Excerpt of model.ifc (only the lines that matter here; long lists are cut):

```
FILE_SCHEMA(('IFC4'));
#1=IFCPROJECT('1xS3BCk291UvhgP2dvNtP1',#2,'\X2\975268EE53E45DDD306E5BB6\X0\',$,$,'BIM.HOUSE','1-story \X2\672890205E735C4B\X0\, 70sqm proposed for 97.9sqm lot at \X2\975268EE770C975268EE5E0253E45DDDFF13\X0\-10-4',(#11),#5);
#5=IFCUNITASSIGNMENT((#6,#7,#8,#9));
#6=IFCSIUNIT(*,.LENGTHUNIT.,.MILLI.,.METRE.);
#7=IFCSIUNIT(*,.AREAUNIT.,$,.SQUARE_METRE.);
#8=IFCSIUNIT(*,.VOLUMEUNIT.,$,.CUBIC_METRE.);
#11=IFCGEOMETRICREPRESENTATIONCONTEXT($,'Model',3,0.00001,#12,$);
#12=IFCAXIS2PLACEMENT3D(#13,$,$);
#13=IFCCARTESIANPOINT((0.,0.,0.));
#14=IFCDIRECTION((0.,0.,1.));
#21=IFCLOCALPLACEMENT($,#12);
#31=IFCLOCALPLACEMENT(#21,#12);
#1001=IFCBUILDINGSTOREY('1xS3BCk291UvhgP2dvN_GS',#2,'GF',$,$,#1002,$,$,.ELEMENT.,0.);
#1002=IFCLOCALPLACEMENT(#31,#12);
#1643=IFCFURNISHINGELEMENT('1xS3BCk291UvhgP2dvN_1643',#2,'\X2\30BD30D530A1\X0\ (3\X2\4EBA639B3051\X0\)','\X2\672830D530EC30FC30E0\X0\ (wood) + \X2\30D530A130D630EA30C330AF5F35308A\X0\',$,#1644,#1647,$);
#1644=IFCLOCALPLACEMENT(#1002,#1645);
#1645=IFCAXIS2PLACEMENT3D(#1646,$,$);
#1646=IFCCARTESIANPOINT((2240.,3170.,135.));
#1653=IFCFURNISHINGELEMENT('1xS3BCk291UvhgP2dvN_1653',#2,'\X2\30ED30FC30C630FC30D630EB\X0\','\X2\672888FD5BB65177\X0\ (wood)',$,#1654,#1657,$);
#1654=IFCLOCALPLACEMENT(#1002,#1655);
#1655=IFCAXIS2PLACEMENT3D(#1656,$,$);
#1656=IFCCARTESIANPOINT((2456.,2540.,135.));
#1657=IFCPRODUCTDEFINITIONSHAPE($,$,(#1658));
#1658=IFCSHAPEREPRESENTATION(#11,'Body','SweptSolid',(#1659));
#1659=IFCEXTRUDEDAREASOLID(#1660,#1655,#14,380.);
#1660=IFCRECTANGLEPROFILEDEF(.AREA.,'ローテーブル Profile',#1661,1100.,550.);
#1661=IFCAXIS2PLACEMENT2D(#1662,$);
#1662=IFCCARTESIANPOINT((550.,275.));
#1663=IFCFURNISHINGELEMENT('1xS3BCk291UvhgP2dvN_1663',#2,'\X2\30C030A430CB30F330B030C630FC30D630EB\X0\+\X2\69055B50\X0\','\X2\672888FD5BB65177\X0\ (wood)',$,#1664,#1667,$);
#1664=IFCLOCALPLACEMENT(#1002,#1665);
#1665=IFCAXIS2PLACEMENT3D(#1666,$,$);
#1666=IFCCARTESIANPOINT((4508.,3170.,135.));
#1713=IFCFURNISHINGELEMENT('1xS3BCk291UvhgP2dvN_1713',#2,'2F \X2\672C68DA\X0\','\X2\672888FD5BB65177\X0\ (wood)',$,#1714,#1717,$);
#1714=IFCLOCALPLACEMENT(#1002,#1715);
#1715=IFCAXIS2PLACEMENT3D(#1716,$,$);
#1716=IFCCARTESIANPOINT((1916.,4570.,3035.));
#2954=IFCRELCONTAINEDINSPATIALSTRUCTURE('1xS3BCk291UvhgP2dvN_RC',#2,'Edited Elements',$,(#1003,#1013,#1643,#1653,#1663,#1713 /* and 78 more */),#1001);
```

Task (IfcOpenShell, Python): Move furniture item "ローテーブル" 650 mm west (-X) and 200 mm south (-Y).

```python
import ifcopenshell
import ifcopenshell.api.geometry
import ifcopenshell.util.placement

model = ifcopenshell.open("model.ifc")

item = model.by_id(1653)
matrix = ifcopenshell.util.placement.get_local_placement(item.ObjectPlacement)
matrix[0, 3] -= 650.0
matrix[1, 3] -= 200.0
ifcopenshell.api.geometry.edit_object_placement(model, product=item, matrix=matrix, is_si=False)

print(ifcopenshell.util.placement.get_local_placement(item.ObjectPlacement).round(3) + 0.0)

model.write("model_edited.ifc")
```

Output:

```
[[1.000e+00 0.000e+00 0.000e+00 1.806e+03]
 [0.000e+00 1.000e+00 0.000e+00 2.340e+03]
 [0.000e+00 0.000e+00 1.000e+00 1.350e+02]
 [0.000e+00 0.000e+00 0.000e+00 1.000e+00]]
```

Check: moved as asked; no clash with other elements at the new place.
